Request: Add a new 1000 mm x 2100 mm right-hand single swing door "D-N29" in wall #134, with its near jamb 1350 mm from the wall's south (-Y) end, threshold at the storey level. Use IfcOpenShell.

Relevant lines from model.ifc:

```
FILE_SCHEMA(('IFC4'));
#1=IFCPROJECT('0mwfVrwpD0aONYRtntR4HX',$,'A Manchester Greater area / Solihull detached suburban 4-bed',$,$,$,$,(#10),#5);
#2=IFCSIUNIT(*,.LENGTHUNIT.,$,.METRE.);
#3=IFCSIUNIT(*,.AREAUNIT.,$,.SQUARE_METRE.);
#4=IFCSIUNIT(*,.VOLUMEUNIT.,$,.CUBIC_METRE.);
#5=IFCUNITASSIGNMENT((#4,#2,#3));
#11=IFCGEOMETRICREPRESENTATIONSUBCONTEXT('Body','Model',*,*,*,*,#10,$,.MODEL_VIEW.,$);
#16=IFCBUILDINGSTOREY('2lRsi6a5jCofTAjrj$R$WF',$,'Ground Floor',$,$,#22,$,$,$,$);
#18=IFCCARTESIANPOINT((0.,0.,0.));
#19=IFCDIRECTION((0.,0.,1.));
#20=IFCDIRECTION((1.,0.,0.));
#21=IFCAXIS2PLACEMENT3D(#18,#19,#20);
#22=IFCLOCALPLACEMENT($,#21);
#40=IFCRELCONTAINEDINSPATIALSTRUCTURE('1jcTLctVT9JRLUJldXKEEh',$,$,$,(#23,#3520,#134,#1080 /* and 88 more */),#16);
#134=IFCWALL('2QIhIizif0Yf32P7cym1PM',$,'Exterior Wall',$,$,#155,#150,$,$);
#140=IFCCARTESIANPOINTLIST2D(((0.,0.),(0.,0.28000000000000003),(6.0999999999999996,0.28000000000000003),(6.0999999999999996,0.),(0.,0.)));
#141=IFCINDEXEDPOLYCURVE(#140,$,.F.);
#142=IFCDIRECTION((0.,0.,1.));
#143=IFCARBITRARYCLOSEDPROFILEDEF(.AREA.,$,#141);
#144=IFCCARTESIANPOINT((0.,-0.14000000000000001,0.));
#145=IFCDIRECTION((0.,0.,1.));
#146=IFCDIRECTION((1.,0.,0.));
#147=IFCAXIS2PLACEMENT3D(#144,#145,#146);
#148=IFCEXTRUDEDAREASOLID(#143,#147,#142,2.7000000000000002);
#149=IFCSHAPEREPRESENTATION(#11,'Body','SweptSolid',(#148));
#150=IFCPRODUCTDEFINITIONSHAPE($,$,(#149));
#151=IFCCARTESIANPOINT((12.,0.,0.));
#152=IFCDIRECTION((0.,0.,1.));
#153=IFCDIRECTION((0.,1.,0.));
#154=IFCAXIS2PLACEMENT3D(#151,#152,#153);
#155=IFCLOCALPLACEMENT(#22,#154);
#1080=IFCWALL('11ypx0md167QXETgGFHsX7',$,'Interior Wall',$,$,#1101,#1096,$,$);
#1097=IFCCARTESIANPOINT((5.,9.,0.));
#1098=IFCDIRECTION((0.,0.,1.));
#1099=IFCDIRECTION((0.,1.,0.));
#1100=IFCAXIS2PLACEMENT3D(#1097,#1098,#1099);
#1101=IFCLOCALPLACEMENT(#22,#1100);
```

```python
import numpy as np
import ifcopenshell
import ifcopenshell.api.feature
import ifcopenshell.api.geometry
import ifcopenshell.api.root
import ifcopenshell.api.spatial
import ifcopenshell.geom
import ifcopenshell.util.element
import ifcopenshell.util.placement
import ifcopenshell.util.representation
import ifcopenshell.util.shape
import ifcopenshell.util.unit

model = ifcopenshell.open("model.ifc")
unit_scale = ifcopenshell.util.unit.calculate_unit_scale(model)
settings = ifcopenshell.geom.settings()


def volume(element):
    """Net volume in cubic metres, openings subtracted."""
    shape = ifcopenshell.geom.create_shape(settings, element)
    return ifcopenshell.util.shape.get_volume(shape.geometry)


wall = model.by_guid("2QIhIizif0Yf32P7cym1PM")
storey = ifcopenshell.util.element.get_container(wall, ifc_class="IfcBuildingStorey")
context = ifcopenshell.util.representation.get_context(model, "Model", "Body", "MODEL_VIEW")
before = volume(wall)

width, height, from_end, sill = 1, 2.1, 1.35, 0.0  # metres

# The wall runs along its own X axis, and the end named is its -X end.
wall_shape = ifcopenshell.geom.create_shape(settings, wall)
x, y, z = ifcopenshell.util.shape.get_vertices(wall_shape.geometry).T
start = x.min() + from_end
face, thickness = float(y.min()), float(y.max() - y.min())
wall_matrix = ifcopenshell.util.placement.get_local_placement(wall.ObjectPlacement)
level = ifcopenshell.util.placement.get_local_placement(storey.ObjectPlacement)[2, 3]


def in_wall(x, y):
    """Placement at x, y metres in the wall's axes, at sill height."""
    matrix = wall_matrix.copy()
    matrix[:, 3] = wall_matrix @ np.array([x / unit_scale, y / unit_scale, 0.0, 1.0])
    matrix[2, 3] = level + sill / unit_scale
    return matrix


# Opening: a box that overshoots both wall faces by 50 mm.
opening = ifcopenshell.api.root.create_entity(model, ifc_class="IfcOpeningElement", predefined_type="OPENING")
box = ifcopenshell.api.geometry.add_wall_representation(
    model, context=context, length=width, height=height, thickness=thickness + 0.1
)
ifcopenshell.api.geometry.assign_representation(model, product=opening, representation=box)
ifcopenshell.api.geometry.edit_object_placement(model, product=opening, matrix=in_wall(start, face - 0.05), is_si=False)
ifcopenshell.api.feature.add_feature(model, feature=opening, element=wall)

door = ifcopenshell.api.root.create_entity(model, ifc_class="IfcDoor", name="D-N29", predefined_type="DOOR")
door.OverallWidth, door.OverallHeight = width / unit_scale, height / unit_scale
door.OperationType = "SINGLE_SWING_RIGHT"
body = ifcopenshell.api.geometry.add_door_representation(
    model,
    context=context,
    overall_width=door.OverallWidth,
    overall_height=door.OverallHeight,
    operation_type="SINGLE_SWING_RIGHT",
    lining_properties={"LiningDepth": thickness / unit_scale, "ThresholdDepth": thickness / unit_scale},
)
ifcopenshell.api.geometry.assign_representation(model, product=door, representation=body)
ifcopenshell.api.spatial.assign_container(model, products=[door], relating_structure=storey)
ifcopenshell.api.feature.add_filling(model, opening=opening, element=door)

# The lining spans the wall, so the door starts at the wall face.
ifcopenshell.api.geometry.edit_object_placement(model, product=door, matrix=in_wall(start, face), is_si=False)

after = volume(wall)

print(f"wall volume {before:.3f} -> {after:.3f} m3")

model.write("model-out.ifc")
```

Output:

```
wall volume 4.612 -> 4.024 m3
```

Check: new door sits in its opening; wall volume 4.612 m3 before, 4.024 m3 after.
